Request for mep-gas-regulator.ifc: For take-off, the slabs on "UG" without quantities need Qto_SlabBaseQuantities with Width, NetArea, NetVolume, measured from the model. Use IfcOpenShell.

First a look at what the model holds.

```python
import ifcopenshell
import ifcopenshell.util.element
import ifcopenshell.util.unit

model = ifcopenshell.open("mep-gas-regulator.ifc")
print(model.schema)
for unit_type in ("LENGTHUNIT", "AREAUNIT", "VOLUMEUNIT"):
    print(unit_type, ifcopenshell.util.unit.calculate_unit_scale(model, unit_type))
storey = next(s for s in model.by_type("IfcBuildingStorey") if s.Name == "UG")
slabs = [e for e in ifcopenshell.util.element.get_decomposition(storey) if e.is_a("IfcSlab")]
for e in sorted(slabs, key=lambda e: e.id()):
    print(e.id(), e.is_a(), e.Name, list(ifcopenshell.util.element.get_psets(e, qtos_only=True)), sep=" | ")
```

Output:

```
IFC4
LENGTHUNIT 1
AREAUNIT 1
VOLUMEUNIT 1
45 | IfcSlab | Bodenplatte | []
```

```python
import ifcopenshell
import ifcopenshell.api.pset
import ifcopenshell.geom
import ifcopenshell.util.element
import ifcopenshell.util.shape
import ifcopenshell.util.unit

model = ifcopenshell.open("mep-gas-regulator.ifc")
unit_scale = ifcopenshell.util.unit.calculate_unit_scale(model)
area_scale = ifcopenshell.util.unit.calculate_unit_scale(model, "AREAUNIT")
volume_scale = ifcopenshell.util.unit.calculate_unit_scale(model, "VOLUMEUNIT")
settings = ifcopenshell.geom.settings()

storey = next(s for s in model.by_type("IfcBuildingStorey") if s.Name == "UG")
slabs = [e for e in ifcopenshell.util.element.get_decomposition(storey) if e.is_a("IfcSlab")]

for e in sorted(slabs, key=lambda e: e.id()):
    if ifcopenshell.util.element.get_psets(e, qtos_only=True, should_inherit=False):
        continue
    # Geometry comes back in metres, in the element's own axes.
    shape = ifcopenshell.geom.create_shape(settings, e)
    values = {
        "Width": ifcopenshell.util.shape.get_z(shape.geometry) / unit_scale,
        "NetArea": ifcopenshell.util.shape.get_footprint_area(shape.geometry) / area_scale,
        "NetVolume": ifcopenshell.util.shape.get_volume(shape.geometry) / volume_scale,
    }
    qto = ifcopenshell.api.pset.add_qto(model, product=e, name="Qto_SlabBaseQuantities")
    ifcopenshell.api.pset.edit_qto(model, qto=qto, properties=values)
    print(e.id(), {k: round(v, 3) for k, v in values.items()})

model.write("mep-gas-regulator_rev.ifc")
```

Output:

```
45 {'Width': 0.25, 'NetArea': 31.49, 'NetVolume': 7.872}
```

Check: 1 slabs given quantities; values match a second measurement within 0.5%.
